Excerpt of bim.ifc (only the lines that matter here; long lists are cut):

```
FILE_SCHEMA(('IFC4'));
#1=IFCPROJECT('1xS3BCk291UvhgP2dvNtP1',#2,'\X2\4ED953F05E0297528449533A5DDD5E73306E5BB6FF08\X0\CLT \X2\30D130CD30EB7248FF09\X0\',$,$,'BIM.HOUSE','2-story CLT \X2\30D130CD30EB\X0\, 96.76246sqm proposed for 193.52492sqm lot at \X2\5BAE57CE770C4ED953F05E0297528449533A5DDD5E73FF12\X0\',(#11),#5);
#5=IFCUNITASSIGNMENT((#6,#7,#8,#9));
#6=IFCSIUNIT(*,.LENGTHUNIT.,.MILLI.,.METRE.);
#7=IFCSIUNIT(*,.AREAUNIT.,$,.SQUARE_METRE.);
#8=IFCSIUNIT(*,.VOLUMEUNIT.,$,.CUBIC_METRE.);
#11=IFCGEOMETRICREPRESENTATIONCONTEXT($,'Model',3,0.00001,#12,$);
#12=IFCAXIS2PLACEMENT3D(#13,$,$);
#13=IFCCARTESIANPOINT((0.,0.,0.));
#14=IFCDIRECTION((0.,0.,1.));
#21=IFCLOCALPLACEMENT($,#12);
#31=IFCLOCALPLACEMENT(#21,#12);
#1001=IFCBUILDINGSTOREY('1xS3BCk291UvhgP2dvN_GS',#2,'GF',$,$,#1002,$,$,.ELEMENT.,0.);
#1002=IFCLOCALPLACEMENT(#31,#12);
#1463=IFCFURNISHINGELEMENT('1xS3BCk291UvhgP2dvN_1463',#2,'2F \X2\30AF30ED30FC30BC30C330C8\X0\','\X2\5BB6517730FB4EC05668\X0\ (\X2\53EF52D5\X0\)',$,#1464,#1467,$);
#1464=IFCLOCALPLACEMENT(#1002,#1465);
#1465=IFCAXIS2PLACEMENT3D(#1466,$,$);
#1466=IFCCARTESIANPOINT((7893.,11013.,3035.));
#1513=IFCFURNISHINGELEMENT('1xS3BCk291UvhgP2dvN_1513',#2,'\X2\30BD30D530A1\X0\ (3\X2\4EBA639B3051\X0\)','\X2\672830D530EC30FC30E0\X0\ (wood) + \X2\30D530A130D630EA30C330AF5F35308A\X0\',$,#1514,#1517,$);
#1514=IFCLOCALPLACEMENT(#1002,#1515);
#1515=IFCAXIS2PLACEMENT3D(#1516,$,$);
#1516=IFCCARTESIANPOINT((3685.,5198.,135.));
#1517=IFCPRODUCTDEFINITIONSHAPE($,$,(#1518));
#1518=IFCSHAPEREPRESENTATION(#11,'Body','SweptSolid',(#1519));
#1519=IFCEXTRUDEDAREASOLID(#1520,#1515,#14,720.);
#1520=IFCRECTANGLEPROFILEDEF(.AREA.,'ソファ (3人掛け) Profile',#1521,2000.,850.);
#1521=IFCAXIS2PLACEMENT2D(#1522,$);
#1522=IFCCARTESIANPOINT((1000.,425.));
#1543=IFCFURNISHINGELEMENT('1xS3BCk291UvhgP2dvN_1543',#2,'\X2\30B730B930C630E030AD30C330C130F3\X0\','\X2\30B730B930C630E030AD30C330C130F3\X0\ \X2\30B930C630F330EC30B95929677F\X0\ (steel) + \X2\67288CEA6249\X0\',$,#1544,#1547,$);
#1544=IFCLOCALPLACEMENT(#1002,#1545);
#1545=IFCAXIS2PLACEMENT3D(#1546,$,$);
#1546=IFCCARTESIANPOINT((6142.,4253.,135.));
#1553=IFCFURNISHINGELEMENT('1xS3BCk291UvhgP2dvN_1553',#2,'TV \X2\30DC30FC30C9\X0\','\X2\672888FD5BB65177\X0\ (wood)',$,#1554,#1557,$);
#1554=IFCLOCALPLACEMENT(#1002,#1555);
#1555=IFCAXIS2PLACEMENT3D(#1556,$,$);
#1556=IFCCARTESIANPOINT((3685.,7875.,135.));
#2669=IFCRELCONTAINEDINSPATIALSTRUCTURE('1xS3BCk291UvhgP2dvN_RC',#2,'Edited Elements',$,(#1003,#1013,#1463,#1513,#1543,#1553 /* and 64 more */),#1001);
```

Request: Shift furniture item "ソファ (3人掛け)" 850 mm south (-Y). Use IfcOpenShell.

```python
import ifcopenshell
import ifcopenshell.api.geometry
import ifcopenshell.util.placement
import ifcopenshell.util.unit

model = ifcopenshell.open("bim.ifc")
unit_scale = ifcopenshell.util.unit.calculate_unit_scale(model)

item = model.by_guid("1xS3BCk291UvhgP2dvN_1513")
matrix = ifcopenshell.util.placement.get_local_placement(item.ObjectPlacement)
matrix[1, 3] -= 0.85 / unit_scale
ifcopenshell.api.geometry.edit_object_placement(model, product=item, matrix=matrix, is_si=False)

print(ifcopenshell.util.placement.get_local_placement(item.ObjectPlacement).round(3) + 0.0)

model.write("bim_updated.ifc")
```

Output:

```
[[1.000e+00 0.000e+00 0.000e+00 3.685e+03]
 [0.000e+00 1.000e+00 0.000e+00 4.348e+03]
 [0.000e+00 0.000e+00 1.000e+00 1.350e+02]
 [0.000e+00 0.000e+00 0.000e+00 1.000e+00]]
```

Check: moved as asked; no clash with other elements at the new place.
